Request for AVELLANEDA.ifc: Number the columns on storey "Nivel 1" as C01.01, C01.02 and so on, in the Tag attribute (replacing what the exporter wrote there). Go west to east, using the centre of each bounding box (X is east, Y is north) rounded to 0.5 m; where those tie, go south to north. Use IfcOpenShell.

First a look at what the model holds.

```python
import ifcopenshell
import ifcopenshell.util.element
import ifcopenshell.util.placement

model = ifcopenshell.open("AVELLANEDA.ifc")
print(model.schema)
storey = next(s for s in model.by_type("IfcBuildingStorey") if s.Name == "Nivel 1")
columns = [e for e in ifcopenshell.util.element.get_decomposition(storey) if e.is_a("IfcColumn")]
for e in sorted(columns, key=lambda e: e.id()):
    origin = ifcopenshell.util.placement.get_local_placement(e.ObjectPlacement)[:3, 3]
    print(e.id(), e.Tag, e.Name, origin.round(2) + 0.0, sep=" | ")
```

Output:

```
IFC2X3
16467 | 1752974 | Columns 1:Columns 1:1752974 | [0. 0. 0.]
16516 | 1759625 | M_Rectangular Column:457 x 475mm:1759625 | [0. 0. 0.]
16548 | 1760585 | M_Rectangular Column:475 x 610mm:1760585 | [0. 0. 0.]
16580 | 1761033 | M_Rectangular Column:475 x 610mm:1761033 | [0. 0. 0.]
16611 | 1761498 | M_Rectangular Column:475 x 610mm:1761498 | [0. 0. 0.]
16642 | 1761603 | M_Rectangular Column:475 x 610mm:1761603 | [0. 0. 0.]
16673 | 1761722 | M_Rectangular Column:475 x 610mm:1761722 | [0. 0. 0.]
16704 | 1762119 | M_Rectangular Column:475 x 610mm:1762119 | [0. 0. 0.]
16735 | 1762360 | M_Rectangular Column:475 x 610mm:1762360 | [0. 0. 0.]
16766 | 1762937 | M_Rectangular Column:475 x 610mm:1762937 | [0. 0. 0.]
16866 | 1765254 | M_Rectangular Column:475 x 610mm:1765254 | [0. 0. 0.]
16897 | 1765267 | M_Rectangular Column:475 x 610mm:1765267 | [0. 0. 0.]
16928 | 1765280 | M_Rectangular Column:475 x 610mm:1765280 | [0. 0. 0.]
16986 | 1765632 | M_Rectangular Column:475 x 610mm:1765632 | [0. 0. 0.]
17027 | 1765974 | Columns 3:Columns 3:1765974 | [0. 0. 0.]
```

```python
import ifcopenshell
import ifcopenshell.geom
import ifcopenshell.util.element
import ifcopenshell.util.shape

model = ifcopenshell.open("AVELLANEDA.ifc")
settings = ifcopenshell.geom.settings()
settings.set("use-world-coords", True)


def centre(element):
    shape = ifcopenshell.geom.create_shape(settings, element)
    return ifcopenshell.util.shape.get_bbox_centroid(shape.geometry)


storey = next(s for s in model.by_type("IfcBuildingStorey") if s.Name == "Nivel 1")
columns = [e for e in ifcopenshell.util.element.get_decomposition(storey) if e.is_a("IfcColumn")]

# Insertion points can sit at a corner or the storey origin, so sort by the geometry (in metres).
centres = {e: centre(e) for e in columns}
columns.sort(key=lambda e: (round(centres[e][0] / 0.5), centres[e][1]))

for i, e in enumerate(columns, start=1):
    number = f"C01.{i:02d}"
    e.Tag = number
    print(e.id(), number)

model.write("AVELLANEDA_edited.ifc")
```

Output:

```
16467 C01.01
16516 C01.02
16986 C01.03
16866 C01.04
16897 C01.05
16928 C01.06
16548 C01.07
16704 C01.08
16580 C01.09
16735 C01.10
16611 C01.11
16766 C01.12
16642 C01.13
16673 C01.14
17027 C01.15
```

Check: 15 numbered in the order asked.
